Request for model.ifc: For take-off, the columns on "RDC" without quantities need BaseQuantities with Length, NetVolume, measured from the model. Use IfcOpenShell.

First a look at what the model holds.

```python
import ifcopenshell
import ifcopenshell.util.element
import ifcopenshell.util.unit

model = ifcopenshell.open("model.ifc")
print(model.schema)
for unit_type in ("LENGTHUNIT", "AREAUNIT", "VOLUMEUNIT"):
    print(unit_type, ifcopenshell.util.unit.calculate_unit_scale(model, unit_type))
storey = next(s for s in model.by_type("IfcBuildingStorey") if s.Name == "RDC")
columns = [e for e in ifcopenshell.util.element.get_decomposition(storey) if e.is_a("IfcColumn")]
for e in sorted(columns, key=lambda e: e.id()):
    print(e.id(), e.is_a(), e.Name, list(ifcopenshell.util.element.get_psets(e, qtos_only=True)), sep=" | ")
```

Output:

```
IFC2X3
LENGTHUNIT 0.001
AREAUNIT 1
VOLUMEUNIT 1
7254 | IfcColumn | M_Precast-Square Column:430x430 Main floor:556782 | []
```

```python
import ifcopenshell
import ifcopenshell.api.pset
import ifcopenshell.geom
import ifcopenshell.util.element
import ifcopenshell.util.shape
import ifcopenshell.util.unit

model = ifcopenshell.open("model.ifc")
unit_scale = ifcopenshell.util.unit.calculate_unit_scale(model)
volume_scale = ifcopenshell.util.unit.calculate_unit_scale(model, "VOLUMEUNIT")
settings = ifcopenshell.geom.settings()

storey = next(s for s in model.by_type("IfcBuildingStorey") if s.Name == "RDC")
columns = [e for e in ifcopenshell.util.element.get_decomposition(storey) if e.is_a("IfcColumn")]

for e in sorted(columns, key=lambda e: e.id()):
    if ifcopenshell.util.element.get_psets(e, qtos_only=True, should_inherit=False):
        continue
    # Geometry comes back in metres, in the element's own axes.
    shape = ifcopenshell.geom.create_shape(settings, e)
    values = {
        "Length": ifcopenshell.util.shape.get_z(shape.geometry) / unit_scale,
        "NetVolume": ifcopenshell.util.shape.get_volume(shape.geometry) / volume_scale,
    }
    qto = ifcopenshell.api.pset.add_qto(model, product=e, name="BaseQuantities")
    ifcopenshell.api.pset.edit_qto(model, qto=qto, properties=values)
    print(e.id(), {k: round(v, 3) for k, v in values.items()})

model.write("model_updated.ifc")
```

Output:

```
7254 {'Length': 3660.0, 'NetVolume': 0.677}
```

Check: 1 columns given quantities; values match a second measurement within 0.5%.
